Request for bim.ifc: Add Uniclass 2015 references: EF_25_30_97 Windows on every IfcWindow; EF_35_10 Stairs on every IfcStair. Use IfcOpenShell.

First a look at what the model holds.

```python
import ifcopenshell

model = ifcopenshell.open("bim.ifc")
print(model.schema)
print("classifications:", [c.Name for c in model.by_type("IfcClassification")])
for ifc_class in ("IfcDoor", "IfcRoof", "IfcStair", "IfcWall", "IfcWindow"):
    print(ifc_class, len(model.by_type(ifc_class)))
```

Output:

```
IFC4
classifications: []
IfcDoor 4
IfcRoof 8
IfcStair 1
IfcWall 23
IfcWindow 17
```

```python
import ifcopenshell
import ifcopenshell.api.classification

model = ifcopenshell.open("bim.ifc")

system = ifcopenshell.api.classification.add_classification(model, classification="Uniclass 2015")

codes = {
    "IfcWindow": ("EF_25_30_97", "Windows"),
    "IfcStair": ("EF_35_10", "Stairs"),
}
for ifc_class, (code, name) in codes.items():
    products = model.by_type(ifc_class)
    ifcopenshell.api.classification.add_reference(
        model, products=products, classification=system, identification=code, name=name
    )
    print(code, len(products))

model.write("bim-out.ifc")
```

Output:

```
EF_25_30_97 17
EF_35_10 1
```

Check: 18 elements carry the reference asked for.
